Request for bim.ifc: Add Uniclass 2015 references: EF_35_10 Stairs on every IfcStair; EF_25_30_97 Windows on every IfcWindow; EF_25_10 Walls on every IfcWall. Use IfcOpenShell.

First a look at what the model holds.

```python
import ifcopenshell

model = ifcopenshell.open("bim.ifc")
print(model.schema)
print("classifications:", [c.Name for c in model.by_type("IfcClassification")])
for ifc_class in ("IfcDoor", "IfcRoof", "IfcStair", "IfcWall", "IfcWindow"):
    print(ifc_class, len(model.by_type(ifc_class)))
```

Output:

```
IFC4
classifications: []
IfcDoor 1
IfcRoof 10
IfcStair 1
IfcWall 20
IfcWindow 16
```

```python
import ifcopenshell
import ifcopenshell.api.classification

model = ifcopenshell.open("bim.ifc")

system = ifcopenshell.api.classification.add_classification(model, classification="Uniclass 2015")

codes = {
    "IfcStair": ("EF_35_10", "Stairs"),
    "IfcWindow": ("EF_25_30_97", "Windows"),
    "IfcWall": ("EF_25_10", "Walls"),
}
for ifc_class, (code, name) in codes.items():
    products = model.by_type(ifc_class)
    ifcopenshell.api.classification.add_reference(
        model, products=products, classification=system, identification=code, name=name
    )
    print(code, len(products))

model.write("bim_v2.ifc")
```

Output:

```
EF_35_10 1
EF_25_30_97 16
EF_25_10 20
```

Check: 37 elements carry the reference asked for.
